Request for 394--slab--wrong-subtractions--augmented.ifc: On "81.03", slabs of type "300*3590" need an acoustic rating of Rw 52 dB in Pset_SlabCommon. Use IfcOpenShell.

First a look at what the model holds.

```python
import ifcopenshell
import ifcopenshell.util.element

model = ifcopenshell.open("394--slab--wrong-subtractions--augmented.ifc")
print(model.schema)
storey = next(s for s in model.by_type("IfcBuildingStorey") if s.Name == "81.03")
slabs = [e for e in ifcopenshell.util.element.get_decomposition(storey) if e.is_a("IfcSlab")]
seen = {}
for e in slabs:
    element_type = ifcopenshell.util.element.get_type(e)
    key = (element_type.Name if element_type != e and element_type else None, ifcopenshell.util.element.get_pset(e, "Pset_SlabCommon", "AcousticRating"))
    seen[key] = seen.get(key, 0) + 1
for (name, value), count in sorted(seen.items(), key=str):
    print(count, "x", name, "|", value)
```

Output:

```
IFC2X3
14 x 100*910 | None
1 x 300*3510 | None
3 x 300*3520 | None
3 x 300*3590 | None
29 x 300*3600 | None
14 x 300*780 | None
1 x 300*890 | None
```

```python
import ifcopenshell
import ifcopenshell.api.pset
import ifcopenshell.util.element

model = ifcopenshell.open("394--slab--wrong-subtractions--augmented.ifc")

storey = next(s for s in model.by_type("IfcBuildingStorey") if s.Name == "81.03")
slabs = [e for e in ifcopenshell.util.element.get_decomposition(storey) if e.is_a("IfcSlab")]

count = 0
for e in slabs:
    element_type = ifcopenshell.util.element.get_type(e)
    if element_type in (None, e) or element_type.Name != "300*3590":
        continue
    found = ifcopenshell.util.element.get_pset(e, "Pset_SlabCommon", should_inherit=False)
    if found:
        pset = model.by_id(found["id"])
        if len(ifcopenshell.util.element.get_elements_by_pset(pset)) > 1:
            pset = ifcopenshell.api.pset.unshare_pset(model, products=[e], pset=pset)[0]
    else:
        pset = ifcopenshell.api.pset.add_pset(model, product=e, name="Pset_SlabCommon")
    ifcopenshell.api.pset.edit_pset(model, pset=pset, properties={"AcousticRating": "Rw 52 dB"})
    count += 1

print(count, "slabs updated")

model.write("394--slab--wrong-subtractions--augmented_v2.ifc")
```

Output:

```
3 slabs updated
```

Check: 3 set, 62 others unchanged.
